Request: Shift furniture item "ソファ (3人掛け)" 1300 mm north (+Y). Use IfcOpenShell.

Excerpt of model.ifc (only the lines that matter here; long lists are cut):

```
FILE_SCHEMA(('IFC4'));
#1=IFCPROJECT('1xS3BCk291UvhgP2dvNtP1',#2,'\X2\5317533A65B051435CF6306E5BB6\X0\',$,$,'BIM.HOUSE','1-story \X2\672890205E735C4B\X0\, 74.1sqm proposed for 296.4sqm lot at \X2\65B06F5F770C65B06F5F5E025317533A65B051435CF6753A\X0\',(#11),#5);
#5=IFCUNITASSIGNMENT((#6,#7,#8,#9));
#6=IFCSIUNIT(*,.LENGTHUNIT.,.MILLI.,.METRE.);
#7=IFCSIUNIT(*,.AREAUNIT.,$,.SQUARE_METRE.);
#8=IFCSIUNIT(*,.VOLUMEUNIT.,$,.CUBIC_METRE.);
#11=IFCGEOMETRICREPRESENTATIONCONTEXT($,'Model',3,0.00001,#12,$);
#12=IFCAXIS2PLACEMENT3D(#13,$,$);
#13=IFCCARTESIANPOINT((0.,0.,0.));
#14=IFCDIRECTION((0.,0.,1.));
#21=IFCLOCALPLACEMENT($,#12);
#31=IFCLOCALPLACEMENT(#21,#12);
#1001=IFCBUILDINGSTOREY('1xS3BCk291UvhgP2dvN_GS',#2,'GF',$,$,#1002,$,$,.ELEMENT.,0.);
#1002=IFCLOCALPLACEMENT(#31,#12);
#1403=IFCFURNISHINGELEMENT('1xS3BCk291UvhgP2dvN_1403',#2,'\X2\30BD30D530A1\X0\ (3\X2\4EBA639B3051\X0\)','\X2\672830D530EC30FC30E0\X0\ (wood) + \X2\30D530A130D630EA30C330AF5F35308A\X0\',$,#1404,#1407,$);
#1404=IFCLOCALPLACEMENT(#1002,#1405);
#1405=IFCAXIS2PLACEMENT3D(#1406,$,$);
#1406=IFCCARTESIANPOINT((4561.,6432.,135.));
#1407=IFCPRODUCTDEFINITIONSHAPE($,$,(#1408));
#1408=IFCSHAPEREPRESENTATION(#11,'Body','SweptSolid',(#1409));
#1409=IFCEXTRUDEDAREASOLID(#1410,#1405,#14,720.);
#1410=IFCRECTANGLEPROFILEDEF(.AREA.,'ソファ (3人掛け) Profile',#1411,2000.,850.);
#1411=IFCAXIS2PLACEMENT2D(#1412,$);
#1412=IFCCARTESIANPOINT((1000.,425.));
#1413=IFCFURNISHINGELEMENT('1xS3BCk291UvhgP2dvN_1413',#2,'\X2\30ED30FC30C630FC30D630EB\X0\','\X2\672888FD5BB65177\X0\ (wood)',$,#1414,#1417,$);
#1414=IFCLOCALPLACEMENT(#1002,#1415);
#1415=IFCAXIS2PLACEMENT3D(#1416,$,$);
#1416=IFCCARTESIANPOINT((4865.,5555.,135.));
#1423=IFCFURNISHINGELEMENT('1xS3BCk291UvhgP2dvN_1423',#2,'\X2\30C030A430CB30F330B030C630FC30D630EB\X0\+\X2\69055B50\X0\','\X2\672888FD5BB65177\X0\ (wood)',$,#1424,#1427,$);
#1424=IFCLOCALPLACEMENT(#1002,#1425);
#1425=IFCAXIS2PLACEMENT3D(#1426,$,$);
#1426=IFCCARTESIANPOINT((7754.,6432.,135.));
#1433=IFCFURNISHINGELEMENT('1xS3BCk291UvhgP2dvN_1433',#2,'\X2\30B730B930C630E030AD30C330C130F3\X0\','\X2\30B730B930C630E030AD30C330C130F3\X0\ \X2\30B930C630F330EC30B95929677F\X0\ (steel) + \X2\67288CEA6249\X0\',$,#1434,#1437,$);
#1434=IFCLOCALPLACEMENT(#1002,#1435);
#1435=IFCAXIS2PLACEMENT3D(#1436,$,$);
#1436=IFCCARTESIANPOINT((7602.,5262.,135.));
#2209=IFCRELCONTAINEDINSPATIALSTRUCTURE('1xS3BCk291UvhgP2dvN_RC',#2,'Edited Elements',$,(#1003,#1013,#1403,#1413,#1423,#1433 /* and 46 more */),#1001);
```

```python
import ifcopenshell
import ifcopenshell.api.geometry
import ifcopenshell.util.placement
import ifcopenshell.util.unit

model = ifcopenshell.open("model.ifc")
unit_scale = ifcopenshell.util.unit.calculate_unit_scale(model)

item = model.by_id(1403)
matrix = ifcopenshell.util.placement.get_local_placement(item.ObjectPlacement)
matrix[1, 3] += 1.3 / unit_scale
ifcopenshell.api.geometry.edit_object_placement(model, product=item, matrix=matrix, is_si=False)

print(ifcopenshell.util.placement.get_local_placement(item.ObjectPlacement).round(3) + 0.0)

model.write("model_updated.ifc")
```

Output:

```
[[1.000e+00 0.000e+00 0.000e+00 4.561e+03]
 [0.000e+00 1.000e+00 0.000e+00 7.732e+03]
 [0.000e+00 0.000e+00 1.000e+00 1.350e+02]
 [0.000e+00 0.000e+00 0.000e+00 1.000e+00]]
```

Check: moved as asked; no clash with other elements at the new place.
